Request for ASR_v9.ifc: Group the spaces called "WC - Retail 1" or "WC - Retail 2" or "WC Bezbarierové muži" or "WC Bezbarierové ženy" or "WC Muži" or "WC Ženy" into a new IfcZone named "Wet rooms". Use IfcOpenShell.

First a look at what the model holds.

```python
import ifcopenshell

model = ifcopenshell.open("ASR_v9.ifc")
print(model.schema)
seen = {}
for space in model.by_type("IfcSpace"):
    seen[space.LongName] = seen.get(space.LongName, 0) + 1
for name, count in sorted(seen.items(), key=str):
    print(count, "x", name)
print("zones:", [z.Name for z in model.by_type("IfcZone")][:20])
```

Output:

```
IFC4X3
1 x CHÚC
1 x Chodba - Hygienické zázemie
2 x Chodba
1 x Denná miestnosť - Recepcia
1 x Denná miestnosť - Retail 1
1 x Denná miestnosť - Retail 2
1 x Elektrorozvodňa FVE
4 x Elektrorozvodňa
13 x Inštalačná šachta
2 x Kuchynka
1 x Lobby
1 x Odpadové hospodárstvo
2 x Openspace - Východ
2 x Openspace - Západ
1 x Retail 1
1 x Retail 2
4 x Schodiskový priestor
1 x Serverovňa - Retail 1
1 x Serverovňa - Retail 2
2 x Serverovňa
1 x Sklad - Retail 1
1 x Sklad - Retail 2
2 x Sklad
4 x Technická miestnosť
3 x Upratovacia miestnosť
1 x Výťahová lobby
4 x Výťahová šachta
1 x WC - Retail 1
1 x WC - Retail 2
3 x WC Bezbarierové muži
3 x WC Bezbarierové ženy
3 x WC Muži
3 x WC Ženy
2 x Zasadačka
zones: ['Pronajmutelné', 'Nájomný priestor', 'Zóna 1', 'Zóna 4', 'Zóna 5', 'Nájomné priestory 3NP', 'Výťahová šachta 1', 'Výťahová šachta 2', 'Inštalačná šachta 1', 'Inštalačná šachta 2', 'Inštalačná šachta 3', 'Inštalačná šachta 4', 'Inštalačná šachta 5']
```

```python
import ifcopenshell
import ifcopenshell.api.group
import ifcopenshell.api.root

model = ifcopenshell.open("ASR_v9.ifc")

names = {"WC - Retail 1", "WC - Retail 2", "WC Bezbarierové muži", "WC Bezbarierové ženy", "WC Muži", "WC Ženy"}
spaces = [s for s in model.by_type("IfcSpace") if s.LongName in names]

zone = ifcopenshell.api.root.create_entity(model, ifc_class="IfcZone", name="Wet rooms")
ifcopenshell.api.group.assign_group(model, products=spaces, group=zone)
print(len(spaces), "spaces in", zone.Name)

model.write("ASR_v9_v2.ifc")
```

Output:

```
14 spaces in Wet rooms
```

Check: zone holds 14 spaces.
